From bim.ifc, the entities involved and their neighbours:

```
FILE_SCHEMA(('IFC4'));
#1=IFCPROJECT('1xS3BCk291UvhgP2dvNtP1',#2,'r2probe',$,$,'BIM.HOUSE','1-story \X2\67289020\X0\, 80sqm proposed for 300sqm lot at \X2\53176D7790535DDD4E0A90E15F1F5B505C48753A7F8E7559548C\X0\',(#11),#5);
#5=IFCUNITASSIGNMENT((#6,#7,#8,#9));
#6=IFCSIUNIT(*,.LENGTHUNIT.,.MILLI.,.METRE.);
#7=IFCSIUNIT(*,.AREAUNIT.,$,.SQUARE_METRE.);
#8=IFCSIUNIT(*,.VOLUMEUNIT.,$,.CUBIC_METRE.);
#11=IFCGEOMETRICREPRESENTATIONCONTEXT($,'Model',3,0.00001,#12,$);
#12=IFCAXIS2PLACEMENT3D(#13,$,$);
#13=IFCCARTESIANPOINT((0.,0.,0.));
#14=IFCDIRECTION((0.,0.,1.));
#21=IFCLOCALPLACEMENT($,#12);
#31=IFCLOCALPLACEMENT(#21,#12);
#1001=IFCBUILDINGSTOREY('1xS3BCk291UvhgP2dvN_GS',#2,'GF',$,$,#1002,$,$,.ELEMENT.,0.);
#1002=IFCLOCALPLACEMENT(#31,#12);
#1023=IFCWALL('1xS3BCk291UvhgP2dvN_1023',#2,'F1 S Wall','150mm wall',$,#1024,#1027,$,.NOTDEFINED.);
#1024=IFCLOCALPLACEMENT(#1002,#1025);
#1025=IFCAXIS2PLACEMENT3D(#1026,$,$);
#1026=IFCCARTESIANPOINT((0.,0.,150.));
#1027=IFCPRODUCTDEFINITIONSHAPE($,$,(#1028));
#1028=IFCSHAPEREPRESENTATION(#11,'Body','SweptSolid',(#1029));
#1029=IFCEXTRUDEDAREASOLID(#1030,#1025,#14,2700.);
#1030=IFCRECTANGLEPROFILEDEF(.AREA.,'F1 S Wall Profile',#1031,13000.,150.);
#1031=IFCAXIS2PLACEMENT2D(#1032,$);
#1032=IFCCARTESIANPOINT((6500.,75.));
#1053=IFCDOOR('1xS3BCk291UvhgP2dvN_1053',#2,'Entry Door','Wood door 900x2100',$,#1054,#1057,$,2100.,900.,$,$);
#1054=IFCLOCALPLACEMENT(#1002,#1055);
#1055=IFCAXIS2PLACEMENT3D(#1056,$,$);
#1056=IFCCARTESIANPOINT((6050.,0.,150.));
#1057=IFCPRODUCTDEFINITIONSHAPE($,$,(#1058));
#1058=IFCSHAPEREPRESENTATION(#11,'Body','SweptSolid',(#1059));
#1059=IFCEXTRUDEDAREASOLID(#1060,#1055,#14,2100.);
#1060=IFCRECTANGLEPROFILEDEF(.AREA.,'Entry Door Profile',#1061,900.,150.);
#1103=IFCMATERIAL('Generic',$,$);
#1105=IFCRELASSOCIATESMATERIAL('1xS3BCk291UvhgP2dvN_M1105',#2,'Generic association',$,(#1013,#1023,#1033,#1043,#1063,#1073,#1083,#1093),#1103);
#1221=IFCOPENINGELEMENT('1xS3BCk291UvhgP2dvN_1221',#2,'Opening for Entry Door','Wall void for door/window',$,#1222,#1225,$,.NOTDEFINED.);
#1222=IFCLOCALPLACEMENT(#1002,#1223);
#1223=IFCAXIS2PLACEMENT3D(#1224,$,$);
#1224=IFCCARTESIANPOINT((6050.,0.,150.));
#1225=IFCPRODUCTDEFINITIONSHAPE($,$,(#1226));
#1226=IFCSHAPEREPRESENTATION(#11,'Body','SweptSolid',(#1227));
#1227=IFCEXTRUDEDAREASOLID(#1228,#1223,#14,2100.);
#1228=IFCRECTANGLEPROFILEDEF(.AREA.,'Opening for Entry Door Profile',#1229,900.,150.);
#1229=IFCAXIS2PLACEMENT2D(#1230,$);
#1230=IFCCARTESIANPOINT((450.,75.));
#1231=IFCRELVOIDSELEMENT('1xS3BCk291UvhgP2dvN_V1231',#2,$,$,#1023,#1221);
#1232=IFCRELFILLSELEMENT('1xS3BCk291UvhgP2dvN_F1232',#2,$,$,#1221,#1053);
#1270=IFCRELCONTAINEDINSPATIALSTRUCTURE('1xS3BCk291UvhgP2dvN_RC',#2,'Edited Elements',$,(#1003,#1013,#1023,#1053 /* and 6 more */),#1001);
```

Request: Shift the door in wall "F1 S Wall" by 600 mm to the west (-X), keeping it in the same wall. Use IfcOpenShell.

```python
import ifcopenshell
import ifcopenshell.api.geometry
import ifcopenshell.util.placement

model = ifcopenshell.open("bim.ifc")

door = model.by_guid("1xS3BCk291UvhgP2dvN_1053")
opening = door.FillsVoids[0].RelatingOpeningElement
wall = opening.VoidsElements[0].RelatingBuildingElement

wall_matrix = ifcopenshell.util.placement.get_local_placement(wall.ObjectPlacement)
shift = wall_matrix[:3, 0] * -600.0
before = ifcopenshell.util.placement.get_local_placement(door.ObjectPlacement)[:3, 3].copy()

# The door is not placed relative to its opening, so move both.
for product in (opening, door):
    matrix = ifcopenshell.util.placement.get_local_placement(product.ObjectPlacement)
    matrix[:3, 3] += shift
    ifcopenshell.api.geometry.edit_object_placement(model, product=product, matrix=matrix, is_si=False)

after = ifcopenshell.util.placement.get_local_placement(door.ObjectPlacement)[:3, 3]
print("door moved by", (after - before).round(3) + 0.0)

model.write("bim_edited.ifc")
```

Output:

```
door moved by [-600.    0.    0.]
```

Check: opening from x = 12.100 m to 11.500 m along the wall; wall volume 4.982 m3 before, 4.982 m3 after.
